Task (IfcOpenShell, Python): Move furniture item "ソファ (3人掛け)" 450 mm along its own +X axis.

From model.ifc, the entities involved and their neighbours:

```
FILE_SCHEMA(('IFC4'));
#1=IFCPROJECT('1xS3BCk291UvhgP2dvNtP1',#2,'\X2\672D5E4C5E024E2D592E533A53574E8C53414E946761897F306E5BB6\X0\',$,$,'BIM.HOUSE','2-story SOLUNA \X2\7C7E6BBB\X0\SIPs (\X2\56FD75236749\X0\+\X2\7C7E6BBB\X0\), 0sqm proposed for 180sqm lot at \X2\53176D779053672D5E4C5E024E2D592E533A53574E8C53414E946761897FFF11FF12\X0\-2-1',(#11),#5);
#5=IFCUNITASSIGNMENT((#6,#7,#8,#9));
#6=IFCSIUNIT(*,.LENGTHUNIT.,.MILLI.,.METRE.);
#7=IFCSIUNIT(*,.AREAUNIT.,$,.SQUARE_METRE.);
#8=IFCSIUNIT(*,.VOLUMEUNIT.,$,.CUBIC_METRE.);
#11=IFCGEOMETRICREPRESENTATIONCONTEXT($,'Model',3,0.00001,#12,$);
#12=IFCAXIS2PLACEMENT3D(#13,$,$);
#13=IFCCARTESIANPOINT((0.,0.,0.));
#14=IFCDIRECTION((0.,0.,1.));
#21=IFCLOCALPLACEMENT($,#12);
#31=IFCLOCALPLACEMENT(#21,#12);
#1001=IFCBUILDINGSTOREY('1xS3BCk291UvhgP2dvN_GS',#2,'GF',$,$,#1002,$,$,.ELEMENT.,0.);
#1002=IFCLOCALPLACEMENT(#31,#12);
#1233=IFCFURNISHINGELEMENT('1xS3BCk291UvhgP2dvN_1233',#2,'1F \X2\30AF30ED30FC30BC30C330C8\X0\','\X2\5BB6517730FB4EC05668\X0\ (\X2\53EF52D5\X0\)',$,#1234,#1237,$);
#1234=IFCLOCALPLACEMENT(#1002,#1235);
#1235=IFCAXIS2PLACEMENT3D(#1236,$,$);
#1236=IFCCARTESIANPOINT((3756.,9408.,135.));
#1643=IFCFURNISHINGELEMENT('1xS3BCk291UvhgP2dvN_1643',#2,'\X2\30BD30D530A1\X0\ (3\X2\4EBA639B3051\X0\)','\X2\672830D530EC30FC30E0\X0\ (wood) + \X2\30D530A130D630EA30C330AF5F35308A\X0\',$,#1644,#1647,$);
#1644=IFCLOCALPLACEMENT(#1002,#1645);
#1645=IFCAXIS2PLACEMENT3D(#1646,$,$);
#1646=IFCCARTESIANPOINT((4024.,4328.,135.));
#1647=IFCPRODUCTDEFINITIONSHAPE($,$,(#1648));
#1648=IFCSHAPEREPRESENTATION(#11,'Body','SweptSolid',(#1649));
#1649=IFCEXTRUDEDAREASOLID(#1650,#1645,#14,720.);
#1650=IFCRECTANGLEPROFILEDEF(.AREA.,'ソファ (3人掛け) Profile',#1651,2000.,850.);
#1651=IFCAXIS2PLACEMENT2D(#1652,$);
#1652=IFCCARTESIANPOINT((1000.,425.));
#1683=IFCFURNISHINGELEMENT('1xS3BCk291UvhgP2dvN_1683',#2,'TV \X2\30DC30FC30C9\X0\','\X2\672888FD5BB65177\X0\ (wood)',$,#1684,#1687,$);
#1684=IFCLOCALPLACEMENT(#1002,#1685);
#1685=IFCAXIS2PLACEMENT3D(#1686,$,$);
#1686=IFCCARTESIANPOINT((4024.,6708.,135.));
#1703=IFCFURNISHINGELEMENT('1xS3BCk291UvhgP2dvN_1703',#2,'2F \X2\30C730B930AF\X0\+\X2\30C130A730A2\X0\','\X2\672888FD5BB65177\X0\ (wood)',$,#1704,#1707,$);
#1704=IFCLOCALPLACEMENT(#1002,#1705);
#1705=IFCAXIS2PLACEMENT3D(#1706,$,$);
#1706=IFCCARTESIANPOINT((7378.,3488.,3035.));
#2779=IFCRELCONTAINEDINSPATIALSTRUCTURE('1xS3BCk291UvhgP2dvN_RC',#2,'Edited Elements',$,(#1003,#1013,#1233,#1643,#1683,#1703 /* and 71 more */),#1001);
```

```python
import ifcopenshell
import ifcopenshell.api.geometry
import ifcopenshell.util.placement
import ifcopenshell.util.unit

model = ifcopenshell.open("model.ifc")
unit_scale = ifcopenshell.util.unit.calculate_unit_scale(model)

item = model.by_guid("1xS3BCk291UvhgP2dvN_1643")
matrix = ifcopenshell.util.placement.get_local_placement(item.ObjectPlacement)
matrix[:3, 3] += matrix[:3, 0] * 0.45 / unit_scale
ifcopenshell.api.geometry.edit_object_placement(model, product=item, matrix=matrix, is_si=False)

print(ifcopenshell.util.placement.get_local_placement(item.ObjectPlacement).round(3) + 0.0)

model.write("model_updated.ifc")
```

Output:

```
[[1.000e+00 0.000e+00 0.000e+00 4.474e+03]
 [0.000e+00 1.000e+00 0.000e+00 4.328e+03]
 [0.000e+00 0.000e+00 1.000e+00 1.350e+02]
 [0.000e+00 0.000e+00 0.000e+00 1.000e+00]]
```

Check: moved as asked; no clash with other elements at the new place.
